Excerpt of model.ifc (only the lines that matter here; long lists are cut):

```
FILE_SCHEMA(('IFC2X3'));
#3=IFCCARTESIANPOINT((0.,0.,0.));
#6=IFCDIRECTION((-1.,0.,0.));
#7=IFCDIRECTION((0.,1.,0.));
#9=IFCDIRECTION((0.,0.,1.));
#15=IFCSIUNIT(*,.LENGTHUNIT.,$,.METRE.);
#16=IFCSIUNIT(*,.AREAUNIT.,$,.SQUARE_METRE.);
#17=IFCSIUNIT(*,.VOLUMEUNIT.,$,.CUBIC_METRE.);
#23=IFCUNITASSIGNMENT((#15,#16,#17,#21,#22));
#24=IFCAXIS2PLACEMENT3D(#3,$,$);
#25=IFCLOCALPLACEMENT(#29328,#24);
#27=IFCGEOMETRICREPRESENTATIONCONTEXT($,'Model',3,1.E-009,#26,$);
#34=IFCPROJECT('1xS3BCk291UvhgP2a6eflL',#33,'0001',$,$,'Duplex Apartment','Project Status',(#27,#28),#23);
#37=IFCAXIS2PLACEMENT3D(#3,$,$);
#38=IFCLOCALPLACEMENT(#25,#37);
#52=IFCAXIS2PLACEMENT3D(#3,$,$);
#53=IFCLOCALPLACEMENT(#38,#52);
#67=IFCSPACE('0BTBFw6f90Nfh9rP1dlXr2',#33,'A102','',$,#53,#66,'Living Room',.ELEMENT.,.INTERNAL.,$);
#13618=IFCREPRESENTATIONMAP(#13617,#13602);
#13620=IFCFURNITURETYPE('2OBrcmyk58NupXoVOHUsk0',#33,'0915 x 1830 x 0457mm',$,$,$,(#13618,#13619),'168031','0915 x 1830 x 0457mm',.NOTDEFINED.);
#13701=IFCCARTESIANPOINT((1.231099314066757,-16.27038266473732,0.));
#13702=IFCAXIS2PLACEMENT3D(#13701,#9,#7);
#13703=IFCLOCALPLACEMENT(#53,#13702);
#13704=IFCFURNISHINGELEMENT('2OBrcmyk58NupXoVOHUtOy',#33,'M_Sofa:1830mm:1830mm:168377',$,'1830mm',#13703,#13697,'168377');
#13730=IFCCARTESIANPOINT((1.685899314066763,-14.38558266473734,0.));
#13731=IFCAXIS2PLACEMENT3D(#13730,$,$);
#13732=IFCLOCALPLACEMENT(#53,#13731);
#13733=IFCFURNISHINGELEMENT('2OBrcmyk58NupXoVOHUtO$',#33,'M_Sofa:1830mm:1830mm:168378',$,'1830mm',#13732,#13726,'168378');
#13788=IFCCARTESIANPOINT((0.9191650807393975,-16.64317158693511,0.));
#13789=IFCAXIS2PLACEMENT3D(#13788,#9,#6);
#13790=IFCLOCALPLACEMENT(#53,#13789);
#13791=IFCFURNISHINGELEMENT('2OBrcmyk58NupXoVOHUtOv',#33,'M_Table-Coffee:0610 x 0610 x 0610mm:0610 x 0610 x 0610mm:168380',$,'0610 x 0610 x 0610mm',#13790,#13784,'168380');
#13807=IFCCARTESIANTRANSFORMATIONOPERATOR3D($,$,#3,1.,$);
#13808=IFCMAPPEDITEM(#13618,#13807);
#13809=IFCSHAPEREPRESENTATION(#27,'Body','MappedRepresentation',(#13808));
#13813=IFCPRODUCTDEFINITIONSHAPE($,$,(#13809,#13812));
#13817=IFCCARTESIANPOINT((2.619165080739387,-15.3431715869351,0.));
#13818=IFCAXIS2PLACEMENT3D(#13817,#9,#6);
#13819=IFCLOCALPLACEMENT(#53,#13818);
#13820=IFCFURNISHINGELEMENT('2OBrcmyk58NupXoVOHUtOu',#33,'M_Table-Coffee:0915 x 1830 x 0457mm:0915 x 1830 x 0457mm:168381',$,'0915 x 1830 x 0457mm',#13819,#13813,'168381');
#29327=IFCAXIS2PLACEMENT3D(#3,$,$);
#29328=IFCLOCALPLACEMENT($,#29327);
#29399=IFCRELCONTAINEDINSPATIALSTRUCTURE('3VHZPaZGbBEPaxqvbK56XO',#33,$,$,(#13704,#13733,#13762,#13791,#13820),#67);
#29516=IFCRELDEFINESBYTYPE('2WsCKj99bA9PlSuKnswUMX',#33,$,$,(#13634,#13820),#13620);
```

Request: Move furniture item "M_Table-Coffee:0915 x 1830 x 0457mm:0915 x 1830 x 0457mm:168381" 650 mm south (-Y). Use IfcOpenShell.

```python
import ifcopenshell
import ifcopenshell.api.geometry
import ifcopenshell.util.placement

model = ifcopenshell.open("model.ifc")

item = model.by_guid("2OBrcmyk58NupXoVOHUtOu")
matrix = ifcopenshell.util.placement.get_local_placement(item.ObjectPlacement)
matrix[1, 3] -= 0.65
ifcopenshell.api.geometry.edit_object_placement(model, product=item, matrix=matrix, is_si=False)

print(ifcopenshell.util.placement.get_local_placement(item.ObjectPlacement).round(3) + 0.0)

model.write("model-out.ifc")
```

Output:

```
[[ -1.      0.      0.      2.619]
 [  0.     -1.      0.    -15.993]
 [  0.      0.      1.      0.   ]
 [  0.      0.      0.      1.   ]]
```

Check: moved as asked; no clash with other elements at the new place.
